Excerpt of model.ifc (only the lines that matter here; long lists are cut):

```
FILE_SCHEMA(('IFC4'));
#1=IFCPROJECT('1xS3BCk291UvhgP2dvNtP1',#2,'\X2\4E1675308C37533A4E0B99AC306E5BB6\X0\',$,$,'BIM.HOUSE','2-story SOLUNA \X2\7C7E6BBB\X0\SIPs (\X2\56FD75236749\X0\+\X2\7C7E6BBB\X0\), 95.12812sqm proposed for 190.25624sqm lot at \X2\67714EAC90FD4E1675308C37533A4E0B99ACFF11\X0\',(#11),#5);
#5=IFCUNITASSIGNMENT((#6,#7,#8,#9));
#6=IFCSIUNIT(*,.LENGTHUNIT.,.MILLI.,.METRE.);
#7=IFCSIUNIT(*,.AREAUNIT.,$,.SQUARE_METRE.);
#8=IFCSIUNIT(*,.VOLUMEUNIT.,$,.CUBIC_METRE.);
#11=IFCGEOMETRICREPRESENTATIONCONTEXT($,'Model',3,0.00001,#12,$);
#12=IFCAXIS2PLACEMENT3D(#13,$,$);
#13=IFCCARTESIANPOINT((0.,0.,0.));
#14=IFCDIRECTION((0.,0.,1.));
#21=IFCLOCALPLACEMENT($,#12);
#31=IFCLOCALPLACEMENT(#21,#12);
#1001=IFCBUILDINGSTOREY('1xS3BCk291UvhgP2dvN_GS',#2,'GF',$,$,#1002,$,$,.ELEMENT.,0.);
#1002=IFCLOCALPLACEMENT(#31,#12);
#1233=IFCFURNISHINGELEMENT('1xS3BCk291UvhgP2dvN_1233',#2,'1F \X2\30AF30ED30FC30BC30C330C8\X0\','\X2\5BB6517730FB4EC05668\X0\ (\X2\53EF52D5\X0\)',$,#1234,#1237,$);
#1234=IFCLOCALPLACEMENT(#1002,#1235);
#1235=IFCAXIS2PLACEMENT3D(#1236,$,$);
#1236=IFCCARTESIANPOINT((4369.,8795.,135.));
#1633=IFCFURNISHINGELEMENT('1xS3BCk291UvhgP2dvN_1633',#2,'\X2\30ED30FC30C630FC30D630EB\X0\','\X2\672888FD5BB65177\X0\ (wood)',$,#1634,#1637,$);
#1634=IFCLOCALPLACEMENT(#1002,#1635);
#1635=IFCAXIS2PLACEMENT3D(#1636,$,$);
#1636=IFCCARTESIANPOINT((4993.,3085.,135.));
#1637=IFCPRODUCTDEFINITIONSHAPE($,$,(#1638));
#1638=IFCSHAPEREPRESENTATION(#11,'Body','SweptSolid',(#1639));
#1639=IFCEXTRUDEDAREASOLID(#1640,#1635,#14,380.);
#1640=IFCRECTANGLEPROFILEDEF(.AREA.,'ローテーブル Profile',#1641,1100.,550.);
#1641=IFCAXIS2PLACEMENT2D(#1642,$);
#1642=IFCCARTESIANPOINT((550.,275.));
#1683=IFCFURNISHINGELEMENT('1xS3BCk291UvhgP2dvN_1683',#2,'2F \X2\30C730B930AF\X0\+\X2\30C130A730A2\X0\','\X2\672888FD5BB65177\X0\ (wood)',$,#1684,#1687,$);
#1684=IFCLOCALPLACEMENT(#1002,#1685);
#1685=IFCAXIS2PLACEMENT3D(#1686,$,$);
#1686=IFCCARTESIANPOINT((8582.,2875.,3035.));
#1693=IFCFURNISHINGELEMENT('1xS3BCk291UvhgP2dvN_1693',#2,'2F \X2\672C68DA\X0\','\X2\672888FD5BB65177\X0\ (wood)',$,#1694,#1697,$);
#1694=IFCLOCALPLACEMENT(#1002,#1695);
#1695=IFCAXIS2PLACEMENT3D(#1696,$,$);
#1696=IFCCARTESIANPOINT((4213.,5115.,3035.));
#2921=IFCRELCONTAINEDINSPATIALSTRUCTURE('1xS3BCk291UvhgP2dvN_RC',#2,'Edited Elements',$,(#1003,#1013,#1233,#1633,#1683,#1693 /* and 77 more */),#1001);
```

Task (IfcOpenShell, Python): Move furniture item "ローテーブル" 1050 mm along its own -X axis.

```python
import ifcopenshell
import ifcopenshell.api.geometry
import ifcopenshell.util.placement

model = ifcopenshell.open("model.ifc")

item = model.by_guid("1xS3BCk291UvhgP2dvN_1633")
matrix = ifcopenshell.util.placement.get_local_placement(item.ObjectPlacement)
matrix[:3, 3] -= matrix[:3, 0] * 1050.0
ifcopenshell.api.geometry.edit_object_placement(model, product=item, matrix=matrix, is_si=False)

print(ifcopenshell.util.placement.get_local_placement(item.ObjectPlacement).round(3) + 0.0)

model.write("model_edited.ifc")
```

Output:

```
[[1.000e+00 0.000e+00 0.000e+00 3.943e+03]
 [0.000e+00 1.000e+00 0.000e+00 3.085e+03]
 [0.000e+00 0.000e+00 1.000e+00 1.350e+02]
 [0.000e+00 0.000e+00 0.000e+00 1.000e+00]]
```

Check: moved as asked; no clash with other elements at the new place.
